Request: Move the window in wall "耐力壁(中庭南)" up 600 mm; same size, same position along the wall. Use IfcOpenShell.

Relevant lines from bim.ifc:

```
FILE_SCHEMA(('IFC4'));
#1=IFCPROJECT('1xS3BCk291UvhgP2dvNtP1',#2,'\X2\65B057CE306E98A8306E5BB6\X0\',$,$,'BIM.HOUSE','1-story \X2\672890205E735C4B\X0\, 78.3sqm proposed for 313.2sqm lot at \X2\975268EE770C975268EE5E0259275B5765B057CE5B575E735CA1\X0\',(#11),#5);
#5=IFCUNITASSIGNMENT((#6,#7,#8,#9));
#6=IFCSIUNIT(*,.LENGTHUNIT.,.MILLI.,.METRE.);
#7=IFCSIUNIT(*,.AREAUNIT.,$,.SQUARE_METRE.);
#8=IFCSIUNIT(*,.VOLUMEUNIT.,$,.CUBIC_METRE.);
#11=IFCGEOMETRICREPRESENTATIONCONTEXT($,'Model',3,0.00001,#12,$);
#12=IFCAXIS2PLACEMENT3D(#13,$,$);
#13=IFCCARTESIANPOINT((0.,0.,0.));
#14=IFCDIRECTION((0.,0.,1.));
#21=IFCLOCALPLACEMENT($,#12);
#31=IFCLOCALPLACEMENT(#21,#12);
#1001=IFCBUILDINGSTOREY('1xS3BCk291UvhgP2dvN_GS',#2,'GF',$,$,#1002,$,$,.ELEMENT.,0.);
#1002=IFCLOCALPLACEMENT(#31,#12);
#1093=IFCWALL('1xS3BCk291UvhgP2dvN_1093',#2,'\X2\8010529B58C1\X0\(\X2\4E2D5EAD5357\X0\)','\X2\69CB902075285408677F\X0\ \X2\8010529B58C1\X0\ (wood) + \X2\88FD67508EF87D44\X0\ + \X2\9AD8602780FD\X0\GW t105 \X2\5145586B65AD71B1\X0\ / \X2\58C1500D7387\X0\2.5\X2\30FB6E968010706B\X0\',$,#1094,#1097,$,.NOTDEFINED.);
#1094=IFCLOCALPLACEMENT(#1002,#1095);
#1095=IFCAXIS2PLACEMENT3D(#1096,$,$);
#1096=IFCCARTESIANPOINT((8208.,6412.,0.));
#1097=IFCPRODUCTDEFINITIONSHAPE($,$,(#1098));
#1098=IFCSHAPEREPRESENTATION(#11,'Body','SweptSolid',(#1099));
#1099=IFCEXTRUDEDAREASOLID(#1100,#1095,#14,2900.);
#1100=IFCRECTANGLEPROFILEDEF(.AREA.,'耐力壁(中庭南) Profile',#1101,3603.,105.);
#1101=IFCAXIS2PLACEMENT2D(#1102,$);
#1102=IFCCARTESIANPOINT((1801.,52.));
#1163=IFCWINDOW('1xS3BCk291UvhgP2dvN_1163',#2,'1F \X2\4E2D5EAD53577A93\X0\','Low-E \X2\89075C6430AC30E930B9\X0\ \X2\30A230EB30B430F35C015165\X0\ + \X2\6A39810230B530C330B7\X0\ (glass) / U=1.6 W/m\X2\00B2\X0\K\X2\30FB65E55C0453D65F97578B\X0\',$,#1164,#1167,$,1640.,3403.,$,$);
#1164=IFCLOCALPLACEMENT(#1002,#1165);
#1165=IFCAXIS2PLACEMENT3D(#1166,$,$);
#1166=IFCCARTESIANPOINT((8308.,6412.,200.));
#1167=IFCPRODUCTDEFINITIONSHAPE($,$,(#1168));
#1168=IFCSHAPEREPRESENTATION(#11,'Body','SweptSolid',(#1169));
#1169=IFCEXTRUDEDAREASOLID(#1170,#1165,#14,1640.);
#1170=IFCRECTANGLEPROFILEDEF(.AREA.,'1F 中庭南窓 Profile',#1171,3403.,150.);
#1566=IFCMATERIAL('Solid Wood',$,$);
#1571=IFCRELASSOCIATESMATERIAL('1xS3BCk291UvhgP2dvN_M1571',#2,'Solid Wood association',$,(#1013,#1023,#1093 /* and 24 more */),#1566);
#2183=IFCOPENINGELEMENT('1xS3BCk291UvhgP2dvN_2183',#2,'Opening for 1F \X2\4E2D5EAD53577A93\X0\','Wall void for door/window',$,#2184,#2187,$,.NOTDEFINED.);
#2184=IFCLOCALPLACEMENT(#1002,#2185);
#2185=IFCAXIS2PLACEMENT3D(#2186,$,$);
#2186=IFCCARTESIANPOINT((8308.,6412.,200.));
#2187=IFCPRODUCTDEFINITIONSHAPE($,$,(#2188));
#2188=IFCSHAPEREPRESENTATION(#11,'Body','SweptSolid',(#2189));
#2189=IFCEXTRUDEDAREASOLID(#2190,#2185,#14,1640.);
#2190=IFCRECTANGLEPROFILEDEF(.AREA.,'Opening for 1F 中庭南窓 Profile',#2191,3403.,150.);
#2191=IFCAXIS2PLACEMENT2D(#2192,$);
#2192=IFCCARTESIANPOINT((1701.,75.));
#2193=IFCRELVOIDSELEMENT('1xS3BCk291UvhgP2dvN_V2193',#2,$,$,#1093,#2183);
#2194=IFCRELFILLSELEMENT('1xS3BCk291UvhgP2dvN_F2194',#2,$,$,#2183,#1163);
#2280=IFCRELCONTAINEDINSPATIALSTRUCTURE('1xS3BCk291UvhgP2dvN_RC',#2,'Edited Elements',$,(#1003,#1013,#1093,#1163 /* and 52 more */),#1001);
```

```python
import numpy as np
import ifcopenshell
import ifcopenshell.api.geometry
import ifcopenshell.util.placement
import ifcopenshell.util.unit

model = ifcopenshell.open("bim.ifc")
unit_scale = ifcopenshell.util.unit.calculate_unit_scale(model)

window = model.by_guid("1xS3BCk291UvhgP2dvN_1163")
opening = window.FillsVoids[0].RelatingOpeningElement
dz = 600.0

shift = np.array([0.0, 0.0, dz])
# The window is not placed relative to its opening, so move both.
for product in (opening, window):
    matrix = ifcopenshell.util.placement.get_local_placement(product.ObjectPlacement)
    matrix[:3, 3] += shift
    ifcopenshell.api.geometry.edit_object_placement(model, product=product, matrix=matrix, is_si=False)

print(f"moved by {dz * unit_scale:+.3f} m")

model.write("bim_v2.ifc")
```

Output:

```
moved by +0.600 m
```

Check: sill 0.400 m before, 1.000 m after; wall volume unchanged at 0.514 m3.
